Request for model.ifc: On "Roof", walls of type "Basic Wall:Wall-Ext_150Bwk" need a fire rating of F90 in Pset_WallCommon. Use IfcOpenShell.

First a look at what the model holds.

```python
import ifcopenshell
import ifcopenshell.util.element

model = ifcopenshell.open("model.ifc")
print(model.schema)
storey = next(s for s in model.by_type("IfcBuildingStorey") if s.Name == "Roof")
walls = [e for e in ifcopenshell.util.element.get_decomposition(storey) if e.is_a("IfcWall")]
seen = {}
for e in walls:
    element_type = ifcopenshell.util.element.get_type(e)
    key = (element_type.Name if element_type != e and element_type else None, ifcopenshell.util.element.get_pset(e, "Pset_WallCommon", "FireRating"))
    seen[key] = seen.get(key, 0) + 1
for (name, value), count in sorted(seen.items(), key=str):
    print(count, "x", name, "|", value)
```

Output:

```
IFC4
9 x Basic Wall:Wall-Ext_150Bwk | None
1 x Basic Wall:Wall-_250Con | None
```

```python
import ifcopenshell
import ifcopenshell.api.pset
import ifcopenshell.util.element

model = ifcopenshell.open("model.ifc")

storey = next(s for s in model.by_type("IfcBuildingStorey") if s.Name == "Roof")
walls = [e for e in ifcopenshell.util.element.get_decomposition(storey) if e.is_a("IfcWall")]

count = 0
for e in walls:
    element_type = ifcopenshell.util.element.get_type(e)
    if element_type in (None, e) or element_type.Name != "Basic Wall:Wall-Ext_150Bwk":
        continue
    # add_pset returns the element's existing set when there is one.
    pset = ifcopenshell.api.pset.add_pset(model, product=e, name="Pset_WallCommon")
    ifcopenshell.api.pset.edit_pset(model, pset=pset, properties={"FireRating": "F90"})
    count += 1

print(count, "walls updated")

model.write("model_v2.ifc")
```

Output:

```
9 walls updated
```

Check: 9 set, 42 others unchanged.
